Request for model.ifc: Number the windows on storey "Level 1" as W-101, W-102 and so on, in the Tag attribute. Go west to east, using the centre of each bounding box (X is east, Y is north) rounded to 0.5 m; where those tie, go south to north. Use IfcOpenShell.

First a look at what the model holds.

```python
import ifcopenshell
import ifcopenshell.util.element
import ifcopenshell.util.placement

model = ifcopenshell.open("model.ifc")
print(model.schema)
storey = next(s for s in model.by_type("IfcBuildingStorey") if s.Name == "Level 1")
windows = [e for e in ifcopenshell.util.element.get_decomposition(storey) if e.is_a("IfcWindow")]
for e in sorted(windows, key=lambda e: e.id()):
    origin = ifcopenshell.util.placement.get_local_placement(e.ObjectPlacement)[:3, 3]
    print(e.id(), e.Tag, e.Name, origin.round(2) + 0.0, sep=" | ")
```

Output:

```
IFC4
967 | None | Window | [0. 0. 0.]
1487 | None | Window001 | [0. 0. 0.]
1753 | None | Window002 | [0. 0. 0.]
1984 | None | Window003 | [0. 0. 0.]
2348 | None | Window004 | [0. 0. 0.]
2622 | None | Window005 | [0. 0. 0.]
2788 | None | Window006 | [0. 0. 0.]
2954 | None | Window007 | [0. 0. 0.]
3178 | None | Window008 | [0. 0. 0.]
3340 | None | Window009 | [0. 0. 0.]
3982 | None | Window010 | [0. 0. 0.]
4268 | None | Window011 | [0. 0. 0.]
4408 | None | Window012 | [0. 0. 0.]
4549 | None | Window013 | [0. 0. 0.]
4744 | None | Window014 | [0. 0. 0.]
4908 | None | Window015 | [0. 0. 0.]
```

```python
import ifcopenshell
import ifcopenshell.geom
import ifcopenshell.util.element
import ifcopenshell.util.shape

model = ifcopenshell.open("model.ifc")
settings = ifcopenshell.geom.settings()
settings.set("use-world-coords", True)


def centre(element):
    shape = ifcopenshell.geom.create_shape(settings, element)
    return ifcopenshell.util.shape.get_bbox_centroid(shape.geometry)


storey = next(s for s in model.by_type("IfcBuildingStorey") if s.Name == "Level 1")
windows = [e for e in ifcopenshell.util.element.get_decomposition(storey) if e.is_a("IfcWindow")]

# Insertion points can sit at a corner or the storey origin, so sort by the geometry (in metres).
centres = {e: centre(e) for e in windows}
windows.sort(key=lambda e: (round(centres[e][0] / 0.5), centres[e][1]))

for i, e in enumerate(windows, start=1):
    number = f"W-1{i:02d}"
    e.Tag = number
    print(e.id(), number)

model.write("model_v2.ifc")
```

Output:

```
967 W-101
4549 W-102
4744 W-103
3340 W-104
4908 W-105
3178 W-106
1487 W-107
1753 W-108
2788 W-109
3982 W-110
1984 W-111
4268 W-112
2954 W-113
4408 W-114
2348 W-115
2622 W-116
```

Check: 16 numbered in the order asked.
